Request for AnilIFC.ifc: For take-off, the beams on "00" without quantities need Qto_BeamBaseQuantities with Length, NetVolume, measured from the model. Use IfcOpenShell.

First a look at what the model holds.

```python
import ifcopenshell
import ifcopenshell.util.element
import ifcopenshell.util.unit

model = ifcopenshell.open("AnilIFC.ifc")
print(model.schema)
for unit_type in ("LENGTHUNIT", "AREAUNIT", "VOLUMEUNIT"):
    print(unit_type, ifcopenshell.util.unit.calculate_unit_scale(model, unit_type))
storey = next(s for s in model.by_type("IfcBuildingStorey") if s.Name == "00")
beams = [e for e in ifcopenshell.util.element.get_decomposition(storey) if e.is_a("IfcBeam")]
for e in sorted(beams, key=lambda e: e.id()):
    print(e.id(), e.is_a(), e.Name, list(ifcopenshell.util.element.get_psets(e, qtos_only=True)), sep=" | ")
```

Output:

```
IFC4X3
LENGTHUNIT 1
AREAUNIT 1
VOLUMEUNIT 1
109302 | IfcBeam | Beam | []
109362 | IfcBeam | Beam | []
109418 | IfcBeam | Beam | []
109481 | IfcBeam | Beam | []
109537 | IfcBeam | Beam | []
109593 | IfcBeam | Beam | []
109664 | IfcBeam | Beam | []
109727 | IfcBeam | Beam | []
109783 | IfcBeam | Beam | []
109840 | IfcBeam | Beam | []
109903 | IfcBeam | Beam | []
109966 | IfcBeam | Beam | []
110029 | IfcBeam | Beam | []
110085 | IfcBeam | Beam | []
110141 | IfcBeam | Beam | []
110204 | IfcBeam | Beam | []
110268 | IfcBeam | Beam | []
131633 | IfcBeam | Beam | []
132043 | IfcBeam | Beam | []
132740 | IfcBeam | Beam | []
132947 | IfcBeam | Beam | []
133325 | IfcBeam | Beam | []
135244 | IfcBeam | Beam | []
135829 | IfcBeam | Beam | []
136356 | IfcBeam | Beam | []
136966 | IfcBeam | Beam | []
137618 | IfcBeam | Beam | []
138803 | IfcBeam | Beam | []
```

```python
import ifcopenshell
import ifcopenshell.api.pset
import ifcopenshell.geom
import ifcopenshell.util.element
import ifcopenshell.util.shape
import ifcopenshell.util.unit

model = ifcopenshell.open("AnilIFC.ifc")
unit_scale = ifcopenshell.util.unit.calculate_unit_scale(model)
volume_scale = ifcopenshell.util.unit.calculate_unit_scale(model, "VOLUMEUNIT")
settings = ifcopenshell.geom.settings()

storey = next(s for s in model.by_type("IfcBuildingStorey") if s.Name == "00")
beams = [e for e in ifcopenshell.util.element.get_decomposition(storey) if e.is_a("IfcBeam")]

for e in sorted(beams, key=lambda e: e.id()):
    if ifcopenshell.util.element.get_psets(e, qtos_only=True, should_inherit=False):
        continue
    # Geometry comes back in metres, in the element's own axes.
    shape = ifcopenshell.geom.create_shape(settings, e)
    values = {
        "Length": ifcopenshell.util.shape.get_max_xyz(shape.geometry) / unit_scale,
        "NetVolume": ifcopenshell.util.shape.get_volume(shape.geometry) / volume_scale,
    }
    qto = ifcopenshell.api.pset.add_qto(model, product=e, name="Qto_BeamBaseQuantities")
    ifcopenshell.api.pset.edit_qto(model, qto=qto, properties=values)
    print(e.id(), {k: round(v, 3) for k, v in values.items()})

model.write("AnilIFC_rev.ifc")
```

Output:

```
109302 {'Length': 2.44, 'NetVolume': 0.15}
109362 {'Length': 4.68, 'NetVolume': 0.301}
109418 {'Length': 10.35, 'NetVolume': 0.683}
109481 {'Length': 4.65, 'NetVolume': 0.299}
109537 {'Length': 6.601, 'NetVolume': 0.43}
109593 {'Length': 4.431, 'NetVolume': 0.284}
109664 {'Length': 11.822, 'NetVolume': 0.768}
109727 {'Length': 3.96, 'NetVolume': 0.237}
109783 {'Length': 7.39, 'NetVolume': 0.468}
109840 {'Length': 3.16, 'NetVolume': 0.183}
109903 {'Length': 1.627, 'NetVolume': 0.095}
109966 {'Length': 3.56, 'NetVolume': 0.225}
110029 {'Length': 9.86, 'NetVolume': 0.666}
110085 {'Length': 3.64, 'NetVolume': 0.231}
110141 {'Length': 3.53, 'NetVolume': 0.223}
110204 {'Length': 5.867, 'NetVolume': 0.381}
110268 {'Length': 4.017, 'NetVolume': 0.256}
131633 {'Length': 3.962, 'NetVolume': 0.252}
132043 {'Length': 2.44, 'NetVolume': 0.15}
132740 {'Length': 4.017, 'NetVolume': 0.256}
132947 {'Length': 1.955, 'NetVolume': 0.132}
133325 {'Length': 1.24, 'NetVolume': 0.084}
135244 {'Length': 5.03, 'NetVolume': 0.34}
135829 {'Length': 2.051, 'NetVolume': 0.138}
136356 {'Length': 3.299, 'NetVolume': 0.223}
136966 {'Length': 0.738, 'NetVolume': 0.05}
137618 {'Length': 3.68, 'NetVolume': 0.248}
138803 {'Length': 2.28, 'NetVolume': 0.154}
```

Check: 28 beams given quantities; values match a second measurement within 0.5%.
